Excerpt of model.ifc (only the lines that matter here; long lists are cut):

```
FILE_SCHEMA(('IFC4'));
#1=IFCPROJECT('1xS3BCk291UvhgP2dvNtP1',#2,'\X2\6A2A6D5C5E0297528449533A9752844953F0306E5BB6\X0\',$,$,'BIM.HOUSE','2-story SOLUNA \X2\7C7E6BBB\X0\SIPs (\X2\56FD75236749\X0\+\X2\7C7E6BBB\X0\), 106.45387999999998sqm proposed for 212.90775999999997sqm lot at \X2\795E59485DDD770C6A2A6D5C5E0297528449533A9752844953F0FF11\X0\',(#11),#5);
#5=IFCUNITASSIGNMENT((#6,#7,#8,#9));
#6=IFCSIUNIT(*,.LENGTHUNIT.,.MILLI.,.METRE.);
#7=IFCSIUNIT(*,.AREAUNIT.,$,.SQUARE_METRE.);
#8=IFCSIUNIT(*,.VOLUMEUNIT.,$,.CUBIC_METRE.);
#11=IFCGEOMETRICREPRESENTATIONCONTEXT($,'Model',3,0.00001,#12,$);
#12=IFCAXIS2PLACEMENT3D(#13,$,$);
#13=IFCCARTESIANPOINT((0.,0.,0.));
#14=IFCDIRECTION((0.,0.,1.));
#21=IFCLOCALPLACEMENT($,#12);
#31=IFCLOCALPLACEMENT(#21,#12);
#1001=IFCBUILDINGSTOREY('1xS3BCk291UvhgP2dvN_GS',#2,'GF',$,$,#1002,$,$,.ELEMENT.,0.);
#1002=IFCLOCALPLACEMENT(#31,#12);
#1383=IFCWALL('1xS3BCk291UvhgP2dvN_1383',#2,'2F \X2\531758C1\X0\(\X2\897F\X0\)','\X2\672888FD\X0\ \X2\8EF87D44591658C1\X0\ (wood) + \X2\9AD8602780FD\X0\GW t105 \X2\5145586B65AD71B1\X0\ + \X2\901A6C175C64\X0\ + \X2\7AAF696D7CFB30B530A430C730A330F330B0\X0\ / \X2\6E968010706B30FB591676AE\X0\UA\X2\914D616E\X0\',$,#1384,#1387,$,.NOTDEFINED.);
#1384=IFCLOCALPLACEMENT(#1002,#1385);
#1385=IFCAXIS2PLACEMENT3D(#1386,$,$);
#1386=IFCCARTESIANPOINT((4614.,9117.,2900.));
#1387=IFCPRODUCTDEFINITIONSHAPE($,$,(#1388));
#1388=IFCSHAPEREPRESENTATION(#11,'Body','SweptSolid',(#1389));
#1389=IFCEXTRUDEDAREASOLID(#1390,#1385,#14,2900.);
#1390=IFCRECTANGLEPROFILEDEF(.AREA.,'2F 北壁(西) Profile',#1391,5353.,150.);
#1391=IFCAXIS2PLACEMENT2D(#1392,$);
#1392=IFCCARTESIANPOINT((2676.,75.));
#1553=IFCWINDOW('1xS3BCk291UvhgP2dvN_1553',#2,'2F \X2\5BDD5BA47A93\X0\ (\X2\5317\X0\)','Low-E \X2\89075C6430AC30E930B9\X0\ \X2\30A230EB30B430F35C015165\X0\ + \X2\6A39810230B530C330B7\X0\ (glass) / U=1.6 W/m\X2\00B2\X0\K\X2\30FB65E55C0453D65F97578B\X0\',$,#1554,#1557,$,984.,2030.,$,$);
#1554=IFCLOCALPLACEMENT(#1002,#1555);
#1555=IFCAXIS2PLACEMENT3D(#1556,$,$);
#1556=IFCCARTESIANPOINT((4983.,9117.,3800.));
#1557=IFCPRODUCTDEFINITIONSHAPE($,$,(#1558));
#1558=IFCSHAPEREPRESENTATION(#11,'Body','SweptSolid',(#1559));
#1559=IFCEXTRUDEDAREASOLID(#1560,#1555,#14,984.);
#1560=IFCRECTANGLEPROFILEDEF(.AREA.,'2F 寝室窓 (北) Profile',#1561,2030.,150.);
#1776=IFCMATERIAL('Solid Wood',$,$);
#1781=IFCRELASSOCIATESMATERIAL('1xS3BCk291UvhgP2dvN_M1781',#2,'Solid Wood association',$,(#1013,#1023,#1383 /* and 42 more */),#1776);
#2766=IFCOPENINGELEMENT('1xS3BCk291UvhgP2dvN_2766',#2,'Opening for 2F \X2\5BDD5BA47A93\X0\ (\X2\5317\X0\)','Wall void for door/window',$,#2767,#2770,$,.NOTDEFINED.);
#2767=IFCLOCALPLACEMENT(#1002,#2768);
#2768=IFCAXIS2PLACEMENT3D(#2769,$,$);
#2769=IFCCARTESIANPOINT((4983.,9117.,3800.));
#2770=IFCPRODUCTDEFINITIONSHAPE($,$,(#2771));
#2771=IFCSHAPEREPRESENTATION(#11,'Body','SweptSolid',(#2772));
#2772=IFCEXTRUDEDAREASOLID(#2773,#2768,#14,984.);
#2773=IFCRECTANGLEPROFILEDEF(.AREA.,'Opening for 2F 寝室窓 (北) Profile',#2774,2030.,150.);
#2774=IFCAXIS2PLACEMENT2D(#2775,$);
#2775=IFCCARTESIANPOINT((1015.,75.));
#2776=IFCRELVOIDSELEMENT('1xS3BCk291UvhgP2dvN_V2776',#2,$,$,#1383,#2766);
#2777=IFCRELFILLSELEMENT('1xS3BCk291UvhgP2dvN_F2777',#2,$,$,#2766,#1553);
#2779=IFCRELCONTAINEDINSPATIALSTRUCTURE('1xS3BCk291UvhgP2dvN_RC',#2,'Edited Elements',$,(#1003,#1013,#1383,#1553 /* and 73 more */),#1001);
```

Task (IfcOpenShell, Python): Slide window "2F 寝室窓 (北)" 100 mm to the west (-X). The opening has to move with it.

```python
import ifcopenshell
import ifcopenshell.api.geometry
import ifcopenshell.util.placement

model = ifcopenshell.open("model.ifc")

window = model.by_guid("1xS3BCk291UvhgP2dvN_1553")
opening = window.FillsVoids[0].RelatingOpeningElement
wall = opening.VoidsElements[0].RelatingBuildingElement

wall_matrix = ifcopenshell.util.placement.get_local_placement(wall.ObjectPlacement)
shift = wall_matrix[:3, 0] * -100.0
before = ifcopenshell.util.placement.get_local_placement(window.ObjectPlacement)[:3, 3].copy()

# The window is not placed relative to its opening, so move both.
for product in (opening, window):
    matrix = ifcopenshell.util.placement.get_local_placement(product.ObjectPlacement)
    matrix[:3, 3] += shift
    ifcopenshell.api.geometry.edit_object_placement(model, product=product, matrix=matrix, is_si=False)

after = ifcopenshell.util.placement.get_local_placement(window.ObjectPlacement)[:3, 3]
print("window moved by", (after - before).round(3) + 0.0)

model.write("model-out.ifc")
```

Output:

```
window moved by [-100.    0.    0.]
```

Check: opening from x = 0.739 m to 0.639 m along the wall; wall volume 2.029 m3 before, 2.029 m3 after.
